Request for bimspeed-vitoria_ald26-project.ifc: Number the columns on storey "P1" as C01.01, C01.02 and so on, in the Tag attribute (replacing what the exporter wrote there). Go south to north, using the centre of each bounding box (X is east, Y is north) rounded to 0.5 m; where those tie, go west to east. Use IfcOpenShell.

First a look at what the model holds.

```python
import ifcopenshell
import ifcopenshell.util.element
import ifcopenshell.util.placement

model = ifcopenshell.open("bimspeed-vitoria_ald26-project.ifc")
print(model.schema)
storey = next(s for s in model.by_type("IfcBuildingStorey") if s.Name == "P1")
columns = [e for e in ifcopenshell.util.element.get_decomposition(storey) if e.is_a("IfcColumn")]
for e in sorted(columns, key=lambda e: e.id()):
    origin = ifcopenshell.util.placement.get_local_placement(e.ObjectPlacement)[:3, 3]
    print(e.id(), e.Tag, e.Name, origin.round(2) + 0.0, sep=" | ")
```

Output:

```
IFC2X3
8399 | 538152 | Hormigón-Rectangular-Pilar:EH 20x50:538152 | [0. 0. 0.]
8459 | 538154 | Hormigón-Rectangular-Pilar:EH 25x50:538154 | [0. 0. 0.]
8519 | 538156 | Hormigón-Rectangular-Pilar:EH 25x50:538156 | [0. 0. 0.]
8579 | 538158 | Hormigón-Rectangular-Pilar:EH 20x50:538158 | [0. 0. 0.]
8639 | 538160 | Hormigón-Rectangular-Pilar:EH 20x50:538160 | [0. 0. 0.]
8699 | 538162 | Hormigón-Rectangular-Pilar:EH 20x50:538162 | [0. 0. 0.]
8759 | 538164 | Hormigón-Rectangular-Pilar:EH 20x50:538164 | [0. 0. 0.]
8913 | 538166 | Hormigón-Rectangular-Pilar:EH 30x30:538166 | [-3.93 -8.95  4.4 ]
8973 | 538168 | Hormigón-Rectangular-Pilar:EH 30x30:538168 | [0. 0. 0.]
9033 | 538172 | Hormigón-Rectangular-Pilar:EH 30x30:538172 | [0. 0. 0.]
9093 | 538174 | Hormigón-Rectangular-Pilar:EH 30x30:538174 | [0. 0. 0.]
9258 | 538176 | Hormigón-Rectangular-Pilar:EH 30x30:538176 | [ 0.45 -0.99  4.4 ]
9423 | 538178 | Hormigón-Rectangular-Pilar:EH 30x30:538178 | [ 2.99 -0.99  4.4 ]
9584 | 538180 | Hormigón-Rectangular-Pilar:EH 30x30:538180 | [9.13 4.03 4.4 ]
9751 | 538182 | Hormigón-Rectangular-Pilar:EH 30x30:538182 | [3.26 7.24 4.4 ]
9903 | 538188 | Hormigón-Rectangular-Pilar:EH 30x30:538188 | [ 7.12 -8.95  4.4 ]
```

```python
import ifcopenshell
import ifcopenshell.geom
import ifcopenshell.util.element
import ifcopenshell.util.shape

model = ifcopenshell.open("bimspeed-vitoria_ald26-project.ifc")
settings = ifcopenshell.geom.settings()
settings.set("use-world-coords", True)


def centre(element):
    shape = ifcopenshell.geom.create_shape(settings, element)
    return ifcopenshell.util.shape.get_bbox_centroid(shape.geometry)


storey = next(s for s in model.by_type("IfcBuildingStorey") if s.Name == "P1")
columns = [e for e in ifcopenshell.util.element.get_decomposition(storey) if e.is_a("IfcColumn")]

# Insertion points can sit at a corner or the storey origin, so sort by the geometry (in metres).
centres = {e: centre(e) for e in columns}
columns.sort(key=lambda e: (round(centres[e][1] / 0.5), centres[e][0]))

for i, e in enumerate(columns, start=1):
    number = f"C01.{i:02d}"
    e.Tag = number
    print(e.id(), number)

model.write("bimspeed-vitoria_ald26-project_updated.ifc")
```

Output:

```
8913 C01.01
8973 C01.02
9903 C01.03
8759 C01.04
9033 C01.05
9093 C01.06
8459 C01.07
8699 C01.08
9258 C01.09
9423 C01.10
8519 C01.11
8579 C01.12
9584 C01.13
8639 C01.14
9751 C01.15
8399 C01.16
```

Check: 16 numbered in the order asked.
